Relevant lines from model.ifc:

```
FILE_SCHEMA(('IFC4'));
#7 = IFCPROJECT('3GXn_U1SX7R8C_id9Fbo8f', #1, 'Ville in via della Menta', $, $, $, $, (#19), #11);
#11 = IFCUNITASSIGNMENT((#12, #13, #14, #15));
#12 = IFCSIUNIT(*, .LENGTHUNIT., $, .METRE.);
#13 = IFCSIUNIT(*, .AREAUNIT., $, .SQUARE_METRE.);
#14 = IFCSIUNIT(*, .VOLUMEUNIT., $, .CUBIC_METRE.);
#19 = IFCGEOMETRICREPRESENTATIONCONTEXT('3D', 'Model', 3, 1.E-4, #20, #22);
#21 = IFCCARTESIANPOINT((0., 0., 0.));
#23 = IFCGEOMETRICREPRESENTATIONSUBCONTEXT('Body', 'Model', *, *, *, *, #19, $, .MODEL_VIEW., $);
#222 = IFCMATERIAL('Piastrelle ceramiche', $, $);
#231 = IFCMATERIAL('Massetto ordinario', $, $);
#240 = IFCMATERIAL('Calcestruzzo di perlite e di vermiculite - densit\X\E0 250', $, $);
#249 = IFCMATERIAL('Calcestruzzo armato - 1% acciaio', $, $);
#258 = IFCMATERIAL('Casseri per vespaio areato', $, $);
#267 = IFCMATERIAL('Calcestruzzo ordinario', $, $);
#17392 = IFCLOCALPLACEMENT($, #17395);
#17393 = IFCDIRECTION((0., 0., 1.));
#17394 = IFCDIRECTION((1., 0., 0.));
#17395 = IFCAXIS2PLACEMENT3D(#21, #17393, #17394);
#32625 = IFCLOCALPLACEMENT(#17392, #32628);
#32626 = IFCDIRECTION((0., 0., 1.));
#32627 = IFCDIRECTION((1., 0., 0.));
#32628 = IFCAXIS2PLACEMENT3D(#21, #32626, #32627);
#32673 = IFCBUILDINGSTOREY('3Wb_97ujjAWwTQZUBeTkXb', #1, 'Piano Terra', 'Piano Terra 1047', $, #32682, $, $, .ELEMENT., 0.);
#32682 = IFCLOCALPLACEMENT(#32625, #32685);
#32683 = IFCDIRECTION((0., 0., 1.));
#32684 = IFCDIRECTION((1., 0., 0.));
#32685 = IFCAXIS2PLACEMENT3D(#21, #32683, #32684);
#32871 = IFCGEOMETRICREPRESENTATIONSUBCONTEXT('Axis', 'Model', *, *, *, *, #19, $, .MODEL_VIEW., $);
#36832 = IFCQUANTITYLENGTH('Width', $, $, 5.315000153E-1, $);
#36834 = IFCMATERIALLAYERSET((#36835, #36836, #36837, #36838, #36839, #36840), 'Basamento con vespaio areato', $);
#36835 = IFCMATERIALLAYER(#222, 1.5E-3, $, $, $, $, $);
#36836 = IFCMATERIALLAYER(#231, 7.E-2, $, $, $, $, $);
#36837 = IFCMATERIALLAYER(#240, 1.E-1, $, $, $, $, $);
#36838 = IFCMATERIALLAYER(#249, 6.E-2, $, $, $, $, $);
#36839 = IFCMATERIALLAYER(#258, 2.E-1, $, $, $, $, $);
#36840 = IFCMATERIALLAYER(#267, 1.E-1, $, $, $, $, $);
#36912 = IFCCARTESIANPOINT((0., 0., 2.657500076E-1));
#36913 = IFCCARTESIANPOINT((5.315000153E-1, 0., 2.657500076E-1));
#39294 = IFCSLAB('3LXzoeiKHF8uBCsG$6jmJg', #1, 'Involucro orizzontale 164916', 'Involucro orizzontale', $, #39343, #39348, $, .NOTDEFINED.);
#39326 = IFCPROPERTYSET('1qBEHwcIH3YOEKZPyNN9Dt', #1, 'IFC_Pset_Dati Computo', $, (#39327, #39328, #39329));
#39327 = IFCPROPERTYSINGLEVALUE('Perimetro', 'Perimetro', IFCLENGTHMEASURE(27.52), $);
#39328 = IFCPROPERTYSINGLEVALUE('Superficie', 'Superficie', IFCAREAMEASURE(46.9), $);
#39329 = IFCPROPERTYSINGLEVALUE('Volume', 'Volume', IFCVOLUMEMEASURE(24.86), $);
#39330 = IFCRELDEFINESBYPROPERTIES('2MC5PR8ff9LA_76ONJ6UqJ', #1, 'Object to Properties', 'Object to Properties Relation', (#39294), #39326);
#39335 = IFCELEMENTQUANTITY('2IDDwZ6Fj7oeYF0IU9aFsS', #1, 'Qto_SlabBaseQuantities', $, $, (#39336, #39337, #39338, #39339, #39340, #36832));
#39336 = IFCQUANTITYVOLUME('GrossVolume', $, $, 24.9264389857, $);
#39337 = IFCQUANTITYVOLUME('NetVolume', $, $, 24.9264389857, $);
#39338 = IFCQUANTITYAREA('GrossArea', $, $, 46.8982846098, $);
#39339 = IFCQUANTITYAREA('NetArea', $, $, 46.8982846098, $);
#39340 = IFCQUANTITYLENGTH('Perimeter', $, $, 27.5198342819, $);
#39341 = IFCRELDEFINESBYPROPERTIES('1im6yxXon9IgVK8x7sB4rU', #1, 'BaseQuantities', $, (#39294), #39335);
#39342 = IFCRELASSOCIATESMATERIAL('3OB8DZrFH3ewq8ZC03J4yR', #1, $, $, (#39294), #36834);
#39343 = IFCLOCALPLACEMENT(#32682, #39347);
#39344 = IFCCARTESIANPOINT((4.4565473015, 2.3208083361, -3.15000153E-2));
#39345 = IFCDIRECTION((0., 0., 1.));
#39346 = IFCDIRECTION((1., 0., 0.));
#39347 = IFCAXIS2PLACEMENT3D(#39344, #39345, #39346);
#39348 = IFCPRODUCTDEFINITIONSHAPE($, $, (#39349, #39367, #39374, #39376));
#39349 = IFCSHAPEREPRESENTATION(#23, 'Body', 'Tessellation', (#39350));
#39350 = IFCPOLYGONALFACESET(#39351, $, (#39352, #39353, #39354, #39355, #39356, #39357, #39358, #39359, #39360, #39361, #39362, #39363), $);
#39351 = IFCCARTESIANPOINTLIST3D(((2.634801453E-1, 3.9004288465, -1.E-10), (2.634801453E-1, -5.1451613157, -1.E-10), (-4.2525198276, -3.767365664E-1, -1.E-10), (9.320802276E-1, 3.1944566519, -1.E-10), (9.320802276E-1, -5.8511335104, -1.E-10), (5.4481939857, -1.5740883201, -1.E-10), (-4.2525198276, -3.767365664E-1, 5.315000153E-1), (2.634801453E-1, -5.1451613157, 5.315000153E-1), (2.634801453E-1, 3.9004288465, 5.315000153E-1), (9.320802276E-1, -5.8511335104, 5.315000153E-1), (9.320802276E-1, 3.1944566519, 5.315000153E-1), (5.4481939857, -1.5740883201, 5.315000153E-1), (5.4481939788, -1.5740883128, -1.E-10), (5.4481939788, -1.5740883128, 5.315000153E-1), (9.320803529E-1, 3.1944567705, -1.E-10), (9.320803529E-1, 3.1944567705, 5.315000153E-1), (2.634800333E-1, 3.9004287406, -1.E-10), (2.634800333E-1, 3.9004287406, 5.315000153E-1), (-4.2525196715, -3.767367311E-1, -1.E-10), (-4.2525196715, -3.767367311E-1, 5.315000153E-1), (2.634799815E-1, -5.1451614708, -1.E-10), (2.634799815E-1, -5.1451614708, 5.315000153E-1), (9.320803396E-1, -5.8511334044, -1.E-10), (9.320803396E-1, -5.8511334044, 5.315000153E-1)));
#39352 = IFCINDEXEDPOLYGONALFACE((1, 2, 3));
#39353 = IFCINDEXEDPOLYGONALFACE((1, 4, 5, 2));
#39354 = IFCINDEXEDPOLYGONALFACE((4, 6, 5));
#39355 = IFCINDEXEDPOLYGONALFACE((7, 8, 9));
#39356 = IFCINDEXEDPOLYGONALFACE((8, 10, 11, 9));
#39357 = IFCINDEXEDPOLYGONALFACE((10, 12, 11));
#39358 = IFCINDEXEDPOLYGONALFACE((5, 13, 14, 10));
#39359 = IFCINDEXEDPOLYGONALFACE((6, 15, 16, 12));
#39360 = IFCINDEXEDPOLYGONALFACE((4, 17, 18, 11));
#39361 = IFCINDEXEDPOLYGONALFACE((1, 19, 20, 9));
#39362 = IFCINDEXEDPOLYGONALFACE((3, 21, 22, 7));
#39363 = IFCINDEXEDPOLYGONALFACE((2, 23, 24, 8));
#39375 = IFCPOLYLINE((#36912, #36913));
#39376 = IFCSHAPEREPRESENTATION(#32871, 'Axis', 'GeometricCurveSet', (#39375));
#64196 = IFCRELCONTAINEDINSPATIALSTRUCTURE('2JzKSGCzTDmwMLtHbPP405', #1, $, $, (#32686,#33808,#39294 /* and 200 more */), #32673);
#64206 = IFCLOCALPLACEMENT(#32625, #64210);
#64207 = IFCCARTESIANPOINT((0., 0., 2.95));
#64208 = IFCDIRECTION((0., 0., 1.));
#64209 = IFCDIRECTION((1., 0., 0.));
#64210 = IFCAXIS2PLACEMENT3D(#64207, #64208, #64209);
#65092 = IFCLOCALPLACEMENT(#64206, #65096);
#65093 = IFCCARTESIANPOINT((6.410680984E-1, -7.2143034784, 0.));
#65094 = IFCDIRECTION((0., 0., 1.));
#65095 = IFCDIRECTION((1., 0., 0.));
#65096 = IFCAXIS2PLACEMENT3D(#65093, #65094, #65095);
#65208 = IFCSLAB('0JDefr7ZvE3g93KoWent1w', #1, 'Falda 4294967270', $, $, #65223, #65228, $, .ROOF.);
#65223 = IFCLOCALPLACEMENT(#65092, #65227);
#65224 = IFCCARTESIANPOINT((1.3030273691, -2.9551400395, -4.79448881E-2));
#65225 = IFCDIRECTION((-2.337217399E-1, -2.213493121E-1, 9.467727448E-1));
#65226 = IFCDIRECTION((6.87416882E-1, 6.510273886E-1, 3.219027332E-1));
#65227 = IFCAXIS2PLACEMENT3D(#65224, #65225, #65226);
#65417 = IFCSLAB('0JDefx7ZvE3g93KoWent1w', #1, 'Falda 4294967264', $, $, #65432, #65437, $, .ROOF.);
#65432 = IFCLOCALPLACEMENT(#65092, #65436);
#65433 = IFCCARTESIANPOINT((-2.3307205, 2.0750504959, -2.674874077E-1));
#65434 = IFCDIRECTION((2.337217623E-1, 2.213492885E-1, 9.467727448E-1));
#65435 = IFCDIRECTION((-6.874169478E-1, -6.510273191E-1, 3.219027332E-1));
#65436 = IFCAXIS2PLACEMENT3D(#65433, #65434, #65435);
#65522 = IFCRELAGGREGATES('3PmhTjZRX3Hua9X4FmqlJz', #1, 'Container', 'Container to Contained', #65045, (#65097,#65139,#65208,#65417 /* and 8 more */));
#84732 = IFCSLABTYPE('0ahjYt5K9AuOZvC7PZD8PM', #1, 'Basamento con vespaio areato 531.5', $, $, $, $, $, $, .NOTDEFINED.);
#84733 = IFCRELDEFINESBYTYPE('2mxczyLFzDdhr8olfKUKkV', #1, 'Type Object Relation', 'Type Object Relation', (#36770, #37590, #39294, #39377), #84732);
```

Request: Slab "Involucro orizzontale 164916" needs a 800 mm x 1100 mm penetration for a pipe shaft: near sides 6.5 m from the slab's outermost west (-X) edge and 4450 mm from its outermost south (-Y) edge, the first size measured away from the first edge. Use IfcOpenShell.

```python
import numpy as np
import ifcopenshell
import ifcopenshell.api.feature
import ifcopenshell.api.geometry
import ifcopenshell.api.pset
import ifcopenshell.api.root
import ifcopenshell.geom
import ifcopenshell.util.element
import ifcopenshell.util.placement
import ifcopenshell.util.representation
import ifcopenshell.util.shape
import ifcopenshell.util.unit

model = ifcopenshell.open("model.ifc")
unit_scale = ifcopenshell.util.unit.calculate_unit_scale(model)
area_scale = ifcopenshell.util.unit.calculate_unit_scale(model, "AREAUNIT")
volume_scale = ifcopenshell.util.unit.calculate_unit_scale(model, "VOLUMEUNIT")
settings = ifcopenshell.geom.settings()


def volume(element):
    """Net volume in cubic metres, openings subtracted."""
    shape = ifcopenshell.geom.create_shape(settings, element)
    return ifcopenshell.util.shape.get_volume(shape.geometry)


slab = model.by_guid("3LXzoeiKHF8uBCsG$6jmJg")
before = volume(slab)

# Extent in the slab's own axes, in metres. The edges named are its -X and -Y sides.
slab_shape = ifcopenshell.geom.create_shape(settings, slab)
vertices = ifcopenshell.util.shape.get_vertices(slab_shape.geometry)
x_min, y_min, bottom = vertices.min(axis=0)
top = vertices[:, 2].max()

opening = ifcopenshell.api.root.create_entity(model, ifc_class="IfcOpeningElement", name="Pipe shaft opening", predefined_type="OPENING")
context = ifcopenshell.util.representation.get_context(model, "Model", "Body", "MODEL_VIEW")
width, depth = 0.8, 1.1
outline = [(0.0, 0.0), (width, 0.0), (width, depth), (0.0, depth), (0.0, 0.0)]
# Overshoot both faces by 50 mm so the cut is clean.
shape = ifcopenshell.api.geometry.add_slab_representation(
    model, context=context, depth=top - bottom + 0.1, polyline=outline
)
ifcopenshell.api.geometry.assign_representation(model, product=opening, representation=shape)

matrix = ifcopenshell.util.placement.get_local_placement(slab.ObjectPlacement)
matrix[:, 3] = matrix @ np.append(np.array([x_min + 6.5, y_min + 4.45, bottom - 0.05]) / unit_scale, 1.0)
ifcopenshell.api.geometry.edit_object_placement(model, product=opening, matrix=matrix, is_si=False)
ifcopenshell.api.feature.add_feature(model, feature=opening, element=slab)

after = volume(slab)

# Update the slab's stored quantities.
pset = model.by_id(ifcopenshell.util.element.get_pset(slab, "IFC_Pset_Dati Computo", should_inherit=False)["id"])
ifcopenshell.api.pset.edit_pset(model, pset=pset, properties={
    "Superficie": model.create_entity("IfcAreaMeasure", after / (top - bottom) / area_scale),
    "Volume": model.create_entity("IfcVolumeMeasure", after / volume_scale),
})
qto = model.by_id(ifcopenshell.util.element.get_pset(slab, "Qto_SlabBaseQuantities", should_inherit=False)["id"])
ifcopenshell.api.pset.edit_qto(model, qto=qto, properties={
    "NetVolume": after / volume_scale,
    "NetArea": after / (top - bottom) / area_scale,
})

print(f"slab volume {before:.3f} -> {after:.3f} m3")

model.write("model_updated.ifc")
```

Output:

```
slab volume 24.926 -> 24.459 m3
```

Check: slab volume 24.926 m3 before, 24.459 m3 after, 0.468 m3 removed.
